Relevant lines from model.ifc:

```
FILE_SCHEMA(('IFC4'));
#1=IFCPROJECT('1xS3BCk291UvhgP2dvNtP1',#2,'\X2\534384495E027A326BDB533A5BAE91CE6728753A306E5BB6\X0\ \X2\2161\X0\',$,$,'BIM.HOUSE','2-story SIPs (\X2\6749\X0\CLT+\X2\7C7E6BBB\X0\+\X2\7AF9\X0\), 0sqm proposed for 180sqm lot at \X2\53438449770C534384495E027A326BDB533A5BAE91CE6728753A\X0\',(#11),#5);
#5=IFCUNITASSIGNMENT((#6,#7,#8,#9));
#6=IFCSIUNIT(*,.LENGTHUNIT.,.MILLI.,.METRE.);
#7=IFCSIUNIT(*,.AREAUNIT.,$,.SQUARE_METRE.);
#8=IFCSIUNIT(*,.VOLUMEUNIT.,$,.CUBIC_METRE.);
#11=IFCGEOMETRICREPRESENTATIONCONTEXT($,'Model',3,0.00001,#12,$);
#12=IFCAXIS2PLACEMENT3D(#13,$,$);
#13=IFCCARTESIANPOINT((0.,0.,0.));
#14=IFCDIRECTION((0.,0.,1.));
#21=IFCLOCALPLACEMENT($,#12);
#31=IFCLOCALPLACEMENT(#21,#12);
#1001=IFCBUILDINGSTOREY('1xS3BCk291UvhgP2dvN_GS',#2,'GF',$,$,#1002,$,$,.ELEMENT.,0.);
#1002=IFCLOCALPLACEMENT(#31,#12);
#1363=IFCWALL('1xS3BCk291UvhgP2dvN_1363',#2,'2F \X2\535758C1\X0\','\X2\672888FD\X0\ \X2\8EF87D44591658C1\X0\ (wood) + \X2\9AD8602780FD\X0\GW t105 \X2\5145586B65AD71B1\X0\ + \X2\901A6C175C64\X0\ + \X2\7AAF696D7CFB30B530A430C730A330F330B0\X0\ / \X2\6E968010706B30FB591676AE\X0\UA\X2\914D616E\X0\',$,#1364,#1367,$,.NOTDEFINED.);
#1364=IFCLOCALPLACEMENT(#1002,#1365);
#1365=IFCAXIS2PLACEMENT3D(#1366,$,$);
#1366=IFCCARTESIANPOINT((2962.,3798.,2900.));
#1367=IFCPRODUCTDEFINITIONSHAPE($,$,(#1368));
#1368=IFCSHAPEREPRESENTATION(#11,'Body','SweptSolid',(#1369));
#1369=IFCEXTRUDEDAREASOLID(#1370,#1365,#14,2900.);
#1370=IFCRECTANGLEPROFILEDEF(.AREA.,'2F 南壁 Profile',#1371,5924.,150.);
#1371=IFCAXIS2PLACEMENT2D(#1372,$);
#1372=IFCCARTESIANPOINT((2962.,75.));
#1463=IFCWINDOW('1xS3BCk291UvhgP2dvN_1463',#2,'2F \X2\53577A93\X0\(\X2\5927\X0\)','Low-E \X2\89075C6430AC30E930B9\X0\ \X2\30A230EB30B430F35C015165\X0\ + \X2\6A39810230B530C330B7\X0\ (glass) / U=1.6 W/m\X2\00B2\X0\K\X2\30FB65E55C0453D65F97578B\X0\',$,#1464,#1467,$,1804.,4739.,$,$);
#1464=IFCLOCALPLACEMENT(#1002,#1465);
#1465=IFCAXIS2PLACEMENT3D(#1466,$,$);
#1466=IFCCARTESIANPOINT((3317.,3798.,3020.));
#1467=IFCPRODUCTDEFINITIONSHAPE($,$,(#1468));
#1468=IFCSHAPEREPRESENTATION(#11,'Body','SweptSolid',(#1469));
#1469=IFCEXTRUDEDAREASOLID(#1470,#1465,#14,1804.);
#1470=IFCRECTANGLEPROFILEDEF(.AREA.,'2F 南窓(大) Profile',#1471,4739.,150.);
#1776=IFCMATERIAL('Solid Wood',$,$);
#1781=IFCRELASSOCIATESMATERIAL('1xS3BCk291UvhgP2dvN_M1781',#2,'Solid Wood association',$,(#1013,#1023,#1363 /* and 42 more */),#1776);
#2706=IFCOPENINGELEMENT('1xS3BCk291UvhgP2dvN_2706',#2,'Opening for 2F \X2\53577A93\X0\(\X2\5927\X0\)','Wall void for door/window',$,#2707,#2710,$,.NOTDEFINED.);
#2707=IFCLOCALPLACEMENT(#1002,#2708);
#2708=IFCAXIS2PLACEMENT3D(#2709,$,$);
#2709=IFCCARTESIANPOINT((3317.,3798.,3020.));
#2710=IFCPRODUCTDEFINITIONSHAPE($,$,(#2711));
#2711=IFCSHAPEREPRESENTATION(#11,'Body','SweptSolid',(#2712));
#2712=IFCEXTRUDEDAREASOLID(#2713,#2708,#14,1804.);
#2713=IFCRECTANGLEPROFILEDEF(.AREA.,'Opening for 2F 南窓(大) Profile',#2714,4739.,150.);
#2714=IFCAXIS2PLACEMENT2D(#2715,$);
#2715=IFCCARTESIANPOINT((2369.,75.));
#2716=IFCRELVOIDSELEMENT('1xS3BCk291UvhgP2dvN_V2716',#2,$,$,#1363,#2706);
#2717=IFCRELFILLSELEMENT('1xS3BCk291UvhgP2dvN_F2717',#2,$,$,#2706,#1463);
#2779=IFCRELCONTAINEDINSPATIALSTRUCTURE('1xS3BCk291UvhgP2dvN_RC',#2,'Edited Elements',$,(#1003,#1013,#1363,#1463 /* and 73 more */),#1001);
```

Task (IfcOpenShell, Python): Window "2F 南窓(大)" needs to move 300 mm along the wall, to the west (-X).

```python
import ifcopenshell
import ifcopenshell.api.geometry
import ifcopenshell.util.placement

model = ifcopenshell.open("model.ifc")

window = model.by_guid("1xS3BCk291UvhgP2dvN_1463")
opening = window.FillsVoids[0].RelatingOpeningElement
wall = opening.VoidsElements[0].RelatingBuildingElement

wall_matrix = ifcopenshell.util.placement.get_local_placement(wall.ObjectPlacement)
shift = wall_matrix[:3, 0] * -300.0
before = ifcopenshell.util.placement.get_local_placement(window.ObjectPlacement)[:3, 3].copy()

# The window is not placed relative to its opening, so move both.
for product in (opening, window):
    matrix = ifcopenshell.util.placement.get_local_placement(product.ObjectPlacement)
    matrix[:3, 3] += shift
    ifcopenshell.api.geometry.edit_object_placement(model, product=product, matrix=matrix, is_si=False)

after = ifcopenshell.util.placement.get_local_placement(window.ObjectPlacement)[:3, 3]
print("window moved by", (after - before).round(3) + 0.0)

model.write("model_updated.ifc")
```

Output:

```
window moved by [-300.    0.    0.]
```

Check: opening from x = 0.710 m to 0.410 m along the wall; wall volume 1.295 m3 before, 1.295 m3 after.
